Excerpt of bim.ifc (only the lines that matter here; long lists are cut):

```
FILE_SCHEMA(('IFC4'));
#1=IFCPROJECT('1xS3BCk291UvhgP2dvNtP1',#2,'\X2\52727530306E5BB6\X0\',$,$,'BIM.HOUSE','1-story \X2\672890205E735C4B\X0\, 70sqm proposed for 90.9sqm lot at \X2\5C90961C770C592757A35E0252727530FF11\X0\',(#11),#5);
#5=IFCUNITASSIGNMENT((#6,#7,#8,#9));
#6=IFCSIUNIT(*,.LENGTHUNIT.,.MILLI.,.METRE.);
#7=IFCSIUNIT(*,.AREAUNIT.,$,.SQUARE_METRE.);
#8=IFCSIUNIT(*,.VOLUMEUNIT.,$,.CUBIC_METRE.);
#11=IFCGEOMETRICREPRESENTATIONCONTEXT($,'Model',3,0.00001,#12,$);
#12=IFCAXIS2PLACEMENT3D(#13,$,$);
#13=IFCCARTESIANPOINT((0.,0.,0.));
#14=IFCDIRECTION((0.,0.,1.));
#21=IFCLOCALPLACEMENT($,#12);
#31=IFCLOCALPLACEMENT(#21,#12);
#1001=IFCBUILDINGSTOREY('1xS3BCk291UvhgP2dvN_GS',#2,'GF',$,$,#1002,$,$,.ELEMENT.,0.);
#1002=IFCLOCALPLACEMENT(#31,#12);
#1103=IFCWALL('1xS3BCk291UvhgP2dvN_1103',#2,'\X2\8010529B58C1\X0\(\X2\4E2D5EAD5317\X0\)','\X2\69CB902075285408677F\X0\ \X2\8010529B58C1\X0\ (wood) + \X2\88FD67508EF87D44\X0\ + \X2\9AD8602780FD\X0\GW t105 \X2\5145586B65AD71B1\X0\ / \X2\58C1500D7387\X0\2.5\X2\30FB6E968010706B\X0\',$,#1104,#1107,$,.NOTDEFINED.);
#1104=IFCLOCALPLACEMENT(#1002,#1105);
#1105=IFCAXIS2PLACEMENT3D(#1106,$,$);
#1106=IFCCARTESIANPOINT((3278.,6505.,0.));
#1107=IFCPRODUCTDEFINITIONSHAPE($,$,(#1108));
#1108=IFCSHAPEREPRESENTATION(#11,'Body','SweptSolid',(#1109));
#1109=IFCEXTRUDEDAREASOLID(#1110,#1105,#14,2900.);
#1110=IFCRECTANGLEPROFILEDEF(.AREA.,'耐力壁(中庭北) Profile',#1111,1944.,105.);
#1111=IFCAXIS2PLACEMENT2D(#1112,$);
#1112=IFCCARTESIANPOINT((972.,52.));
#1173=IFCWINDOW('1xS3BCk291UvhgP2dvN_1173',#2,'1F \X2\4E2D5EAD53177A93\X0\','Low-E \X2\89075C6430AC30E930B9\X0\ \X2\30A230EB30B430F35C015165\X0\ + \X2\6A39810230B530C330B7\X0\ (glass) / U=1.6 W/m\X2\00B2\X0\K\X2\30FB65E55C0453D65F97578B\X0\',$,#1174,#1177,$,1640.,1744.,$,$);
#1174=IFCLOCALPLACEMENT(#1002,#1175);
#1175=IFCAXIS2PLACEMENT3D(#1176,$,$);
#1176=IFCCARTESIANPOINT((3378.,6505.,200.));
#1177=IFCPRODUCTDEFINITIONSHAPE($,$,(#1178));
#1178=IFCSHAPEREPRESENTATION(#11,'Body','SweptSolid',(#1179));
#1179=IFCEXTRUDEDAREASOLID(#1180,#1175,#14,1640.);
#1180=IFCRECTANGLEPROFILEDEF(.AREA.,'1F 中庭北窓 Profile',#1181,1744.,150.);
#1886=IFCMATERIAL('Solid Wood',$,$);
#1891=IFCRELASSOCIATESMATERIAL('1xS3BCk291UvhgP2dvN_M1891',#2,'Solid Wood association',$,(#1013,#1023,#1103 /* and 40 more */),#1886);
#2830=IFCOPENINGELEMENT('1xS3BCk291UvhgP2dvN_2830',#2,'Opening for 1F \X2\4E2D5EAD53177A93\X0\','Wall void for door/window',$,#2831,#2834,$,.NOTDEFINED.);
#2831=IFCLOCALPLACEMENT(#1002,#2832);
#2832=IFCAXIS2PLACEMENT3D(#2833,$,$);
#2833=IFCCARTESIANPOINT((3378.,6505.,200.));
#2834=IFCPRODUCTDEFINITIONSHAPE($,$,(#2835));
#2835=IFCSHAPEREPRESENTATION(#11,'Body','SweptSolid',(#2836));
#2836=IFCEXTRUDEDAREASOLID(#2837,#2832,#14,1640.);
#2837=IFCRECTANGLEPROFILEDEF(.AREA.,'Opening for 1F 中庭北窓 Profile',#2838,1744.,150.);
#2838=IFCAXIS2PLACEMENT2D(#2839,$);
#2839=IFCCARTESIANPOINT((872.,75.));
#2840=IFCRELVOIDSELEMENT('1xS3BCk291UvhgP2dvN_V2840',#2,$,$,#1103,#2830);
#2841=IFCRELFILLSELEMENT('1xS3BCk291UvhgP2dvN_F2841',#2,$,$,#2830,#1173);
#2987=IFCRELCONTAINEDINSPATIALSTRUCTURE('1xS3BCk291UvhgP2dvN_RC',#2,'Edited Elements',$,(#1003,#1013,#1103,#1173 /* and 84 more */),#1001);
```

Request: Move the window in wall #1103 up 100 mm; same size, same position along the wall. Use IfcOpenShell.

```python
import numpy as np
import ifcopenshell
import ifcopenshell.api.geometry
import ifcopenshell.util.placement
import ifcopenshell.util.unit

model = ifcopenshell.open("bim.ifc")
unit_scale = ifcopenshell.util.unit.calculate_unit_scale(model)

window = model.by_guid("1xS3BCk291UvhgP2dvN_1173")
opening = window.FillsVoids[0].RelatingOpeningElement
dz = 0.1 / unit_scale

shift = np.array([0.0, 0.0, dz])
# The window is not placed relative to its opening, so move both.
for product in (opening, window):
    matrix = ifcopenshell.util.placement.get_local_placement(product.ObjectPlacement)
    matrix[:3, 3] += shift
    ifcopenshell.api.geometry.edit_object_placement(model, product=product, matrix=matrix, is_si=False)

print(f"moved by {dz * unit_scale:+.3f} m")

model.write("bim_rev.ifc")
```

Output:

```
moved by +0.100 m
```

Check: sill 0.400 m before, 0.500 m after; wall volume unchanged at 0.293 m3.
